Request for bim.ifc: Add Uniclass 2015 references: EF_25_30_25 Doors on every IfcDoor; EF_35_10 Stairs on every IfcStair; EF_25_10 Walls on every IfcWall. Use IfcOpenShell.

First a look at what the model holds.

```python
import ifcopenshell

model = ifcopenshell.open("bim.ifc")
print(model.schema)
print("classifications:", [c.Name for c in model.by_type("IfcClassification")])
for ifc_class in ("IfcDoor", "IfcRoof", "IfcStair", "IfcWall", "IfcWindow"):
    print(ifc_class, len(model.by_type(ifc_class)))
```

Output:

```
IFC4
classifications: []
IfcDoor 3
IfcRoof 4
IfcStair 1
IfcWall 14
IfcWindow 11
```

```python
import ifcopenshell
import ifcopenshell.api.classification

model = ifcopenshell.open("bim.ifc")

system = ifcopenshell.api.classification.add_classification(model, classification="Uniclass 2015")

codes = {
    "IfcDoor": ("EF_25_30_25", "Doors"),
    "IfcStair": ("EF_35_10", "Stairs"),
    "IfcWall": ("EF_25_10", "Walls"),
}
for ifc_class, (code, name) in codes.items():
    products = model.by_type(ifc_class)
    ifcopenshell.api.classification.add_reference(
        model, products=products, classification=system, identification=code, name=name
    )
    print(code, len(products))

model.write("bim_rev.ifc")
```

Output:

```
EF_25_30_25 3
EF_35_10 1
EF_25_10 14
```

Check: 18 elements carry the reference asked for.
